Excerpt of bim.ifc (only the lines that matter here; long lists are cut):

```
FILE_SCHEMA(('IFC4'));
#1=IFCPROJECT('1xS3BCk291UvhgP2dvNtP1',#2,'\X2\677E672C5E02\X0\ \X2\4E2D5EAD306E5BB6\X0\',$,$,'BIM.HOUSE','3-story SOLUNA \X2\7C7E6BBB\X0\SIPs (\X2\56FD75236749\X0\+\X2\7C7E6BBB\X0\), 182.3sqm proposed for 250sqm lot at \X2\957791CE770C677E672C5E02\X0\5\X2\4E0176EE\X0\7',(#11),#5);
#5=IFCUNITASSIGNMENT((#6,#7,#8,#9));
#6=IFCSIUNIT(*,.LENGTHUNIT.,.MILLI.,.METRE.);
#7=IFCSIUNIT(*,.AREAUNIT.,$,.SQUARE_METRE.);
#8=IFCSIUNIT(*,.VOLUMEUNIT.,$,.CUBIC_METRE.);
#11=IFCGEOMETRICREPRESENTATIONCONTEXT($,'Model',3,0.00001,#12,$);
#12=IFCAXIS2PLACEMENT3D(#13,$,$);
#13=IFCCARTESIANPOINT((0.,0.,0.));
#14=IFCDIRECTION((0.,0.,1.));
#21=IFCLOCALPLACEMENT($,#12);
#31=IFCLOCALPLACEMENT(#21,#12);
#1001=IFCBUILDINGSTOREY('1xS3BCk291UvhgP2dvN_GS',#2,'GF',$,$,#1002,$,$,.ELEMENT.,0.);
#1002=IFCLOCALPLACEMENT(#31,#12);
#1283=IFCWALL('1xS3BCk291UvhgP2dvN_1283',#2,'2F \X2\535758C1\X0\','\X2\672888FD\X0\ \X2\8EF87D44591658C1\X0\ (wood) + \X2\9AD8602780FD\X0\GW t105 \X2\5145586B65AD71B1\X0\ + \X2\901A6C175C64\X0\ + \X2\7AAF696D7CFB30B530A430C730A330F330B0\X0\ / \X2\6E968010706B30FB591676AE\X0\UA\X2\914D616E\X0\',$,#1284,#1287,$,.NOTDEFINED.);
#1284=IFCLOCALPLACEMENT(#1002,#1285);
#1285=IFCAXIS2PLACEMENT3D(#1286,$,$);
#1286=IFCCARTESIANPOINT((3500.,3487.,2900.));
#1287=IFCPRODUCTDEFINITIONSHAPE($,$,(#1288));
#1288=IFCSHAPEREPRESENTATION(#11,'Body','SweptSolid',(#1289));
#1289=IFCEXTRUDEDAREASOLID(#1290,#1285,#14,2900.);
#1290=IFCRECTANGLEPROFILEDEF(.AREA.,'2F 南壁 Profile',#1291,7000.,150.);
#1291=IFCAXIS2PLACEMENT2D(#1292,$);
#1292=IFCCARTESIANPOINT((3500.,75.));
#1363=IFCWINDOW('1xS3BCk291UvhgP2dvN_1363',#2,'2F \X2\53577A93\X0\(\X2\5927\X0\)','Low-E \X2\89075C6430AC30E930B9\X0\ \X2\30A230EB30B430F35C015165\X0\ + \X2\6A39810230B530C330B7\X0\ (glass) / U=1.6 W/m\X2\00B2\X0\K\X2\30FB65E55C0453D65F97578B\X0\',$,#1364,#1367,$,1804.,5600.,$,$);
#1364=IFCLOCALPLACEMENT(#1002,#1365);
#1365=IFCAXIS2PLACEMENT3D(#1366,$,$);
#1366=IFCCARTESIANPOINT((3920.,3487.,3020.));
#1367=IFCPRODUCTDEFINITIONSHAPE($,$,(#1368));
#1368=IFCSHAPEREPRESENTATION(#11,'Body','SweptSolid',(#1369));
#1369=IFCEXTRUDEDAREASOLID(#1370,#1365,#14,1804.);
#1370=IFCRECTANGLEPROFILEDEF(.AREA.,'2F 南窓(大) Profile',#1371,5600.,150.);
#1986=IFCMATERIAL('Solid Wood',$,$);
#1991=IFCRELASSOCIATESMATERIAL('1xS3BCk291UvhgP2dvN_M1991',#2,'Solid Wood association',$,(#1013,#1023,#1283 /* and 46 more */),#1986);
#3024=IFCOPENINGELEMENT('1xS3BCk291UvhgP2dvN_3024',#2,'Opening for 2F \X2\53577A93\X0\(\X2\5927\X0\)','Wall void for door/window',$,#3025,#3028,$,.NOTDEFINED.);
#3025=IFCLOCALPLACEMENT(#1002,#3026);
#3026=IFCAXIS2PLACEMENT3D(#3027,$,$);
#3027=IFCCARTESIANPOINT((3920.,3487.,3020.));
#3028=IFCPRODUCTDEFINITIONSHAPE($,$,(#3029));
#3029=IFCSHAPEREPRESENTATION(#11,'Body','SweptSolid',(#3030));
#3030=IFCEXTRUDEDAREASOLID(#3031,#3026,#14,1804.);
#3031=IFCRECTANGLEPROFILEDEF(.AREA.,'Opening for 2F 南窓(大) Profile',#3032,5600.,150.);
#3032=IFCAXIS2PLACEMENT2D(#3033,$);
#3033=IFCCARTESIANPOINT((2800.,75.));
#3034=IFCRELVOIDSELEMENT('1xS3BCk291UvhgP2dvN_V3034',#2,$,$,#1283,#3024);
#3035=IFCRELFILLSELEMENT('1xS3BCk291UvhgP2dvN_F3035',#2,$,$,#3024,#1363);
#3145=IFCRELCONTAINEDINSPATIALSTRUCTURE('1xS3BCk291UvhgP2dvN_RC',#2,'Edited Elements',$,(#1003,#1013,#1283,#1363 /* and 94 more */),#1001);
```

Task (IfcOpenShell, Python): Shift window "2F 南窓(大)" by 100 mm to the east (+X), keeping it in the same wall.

```python
import ifcopenshell
import ifcopenshell.api.geometry
import ifcopenshell.util.placement
import ifcopenshell.util.unit

model = ifcopenshell.open("bim.ifc")
unit_scale = ifcopenshell.util.unit.calculate_unit_scale(model)

window = model.by_guid("1xS3BCk291UvhgP2dvN_1363")
opening = window.FillsVoids[0].RelatingOpeningElement
wall = opening.VoidsElements[0].RelatingBuildingElement

wall_matrix = ifcopenshell.util.placement.get_local_placement(wall.ObjectPlacement)
shift = wall_matrix[:3, 0] * 0.1 / unit_scale
before = ifcopenshell.util.placement.get_local_placement(window.ObjectPlacement)[:3, 3].copy()

# The window is not placed relative to its opening, so move both.
for product in (opening, window):
    matrix = ifcopenshell.util.placement.get_local_placement(product.ObjectPlacement)
    matrix[:3, 3] += shift
    ifcopenshell.api.geometry.edit_object_placement(model, product=product, matrix=matrix, is_si=False)

after = ifcopenshell.util.placement.get_local_placement(window.ObjectPlacement)[:3, 3]
print("window moved by", (after - before).round(3) + 0.0)

model.write("bim_edited.ifc")
```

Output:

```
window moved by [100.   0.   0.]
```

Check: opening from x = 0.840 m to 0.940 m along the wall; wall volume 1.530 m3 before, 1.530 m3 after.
